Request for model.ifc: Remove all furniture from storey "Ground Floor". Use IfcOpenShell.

First a look at what the model holds.

```python
import ifcopenshell
import ifcopenshell.util.element

model = ifcopenshell.open("model.ifc")
print(model.schema)
storey = next(s for s in model.by_type("IfcBuildingStorey") if s.Name == "Ground Floor")
furniture = [e for e in ifcopenshell.util.element.get_decomposition(storey) if e.is_a("IfcFurnishingElement")]
seen = {}
for e in furniture:
    element_type = ifcopenshell.util.element.get_type(e)
    name = element_type.Name if element_type not in (None, e) else None
    seen[name] = seen.get(name, 0) + 1
for name, count in sorted(seen.items(), key=str):
    print(count, "x", name)
```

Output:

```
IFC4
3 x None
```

```python
import ifcopenshell
import ifcopenshell.api.root
import ifcopenshell.util.element

model = ifcopenshell.open("model.ifc")

storey = next(s for s in model.by_type("IfcBuildingStorey") if s.Name == "Ground Floor")
furniture = [e for e in ifcopenshell.util.element.get_decomposition(storey) if e.is_a("IfcFurnishingElement")]

for e in furniture:
    ifcopenshell.api.root.remove_product(model, product=e)
print(len(furniture), "removed")

model.write("model_updated.ifc")
```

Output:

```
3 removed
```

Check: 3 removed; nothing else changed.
